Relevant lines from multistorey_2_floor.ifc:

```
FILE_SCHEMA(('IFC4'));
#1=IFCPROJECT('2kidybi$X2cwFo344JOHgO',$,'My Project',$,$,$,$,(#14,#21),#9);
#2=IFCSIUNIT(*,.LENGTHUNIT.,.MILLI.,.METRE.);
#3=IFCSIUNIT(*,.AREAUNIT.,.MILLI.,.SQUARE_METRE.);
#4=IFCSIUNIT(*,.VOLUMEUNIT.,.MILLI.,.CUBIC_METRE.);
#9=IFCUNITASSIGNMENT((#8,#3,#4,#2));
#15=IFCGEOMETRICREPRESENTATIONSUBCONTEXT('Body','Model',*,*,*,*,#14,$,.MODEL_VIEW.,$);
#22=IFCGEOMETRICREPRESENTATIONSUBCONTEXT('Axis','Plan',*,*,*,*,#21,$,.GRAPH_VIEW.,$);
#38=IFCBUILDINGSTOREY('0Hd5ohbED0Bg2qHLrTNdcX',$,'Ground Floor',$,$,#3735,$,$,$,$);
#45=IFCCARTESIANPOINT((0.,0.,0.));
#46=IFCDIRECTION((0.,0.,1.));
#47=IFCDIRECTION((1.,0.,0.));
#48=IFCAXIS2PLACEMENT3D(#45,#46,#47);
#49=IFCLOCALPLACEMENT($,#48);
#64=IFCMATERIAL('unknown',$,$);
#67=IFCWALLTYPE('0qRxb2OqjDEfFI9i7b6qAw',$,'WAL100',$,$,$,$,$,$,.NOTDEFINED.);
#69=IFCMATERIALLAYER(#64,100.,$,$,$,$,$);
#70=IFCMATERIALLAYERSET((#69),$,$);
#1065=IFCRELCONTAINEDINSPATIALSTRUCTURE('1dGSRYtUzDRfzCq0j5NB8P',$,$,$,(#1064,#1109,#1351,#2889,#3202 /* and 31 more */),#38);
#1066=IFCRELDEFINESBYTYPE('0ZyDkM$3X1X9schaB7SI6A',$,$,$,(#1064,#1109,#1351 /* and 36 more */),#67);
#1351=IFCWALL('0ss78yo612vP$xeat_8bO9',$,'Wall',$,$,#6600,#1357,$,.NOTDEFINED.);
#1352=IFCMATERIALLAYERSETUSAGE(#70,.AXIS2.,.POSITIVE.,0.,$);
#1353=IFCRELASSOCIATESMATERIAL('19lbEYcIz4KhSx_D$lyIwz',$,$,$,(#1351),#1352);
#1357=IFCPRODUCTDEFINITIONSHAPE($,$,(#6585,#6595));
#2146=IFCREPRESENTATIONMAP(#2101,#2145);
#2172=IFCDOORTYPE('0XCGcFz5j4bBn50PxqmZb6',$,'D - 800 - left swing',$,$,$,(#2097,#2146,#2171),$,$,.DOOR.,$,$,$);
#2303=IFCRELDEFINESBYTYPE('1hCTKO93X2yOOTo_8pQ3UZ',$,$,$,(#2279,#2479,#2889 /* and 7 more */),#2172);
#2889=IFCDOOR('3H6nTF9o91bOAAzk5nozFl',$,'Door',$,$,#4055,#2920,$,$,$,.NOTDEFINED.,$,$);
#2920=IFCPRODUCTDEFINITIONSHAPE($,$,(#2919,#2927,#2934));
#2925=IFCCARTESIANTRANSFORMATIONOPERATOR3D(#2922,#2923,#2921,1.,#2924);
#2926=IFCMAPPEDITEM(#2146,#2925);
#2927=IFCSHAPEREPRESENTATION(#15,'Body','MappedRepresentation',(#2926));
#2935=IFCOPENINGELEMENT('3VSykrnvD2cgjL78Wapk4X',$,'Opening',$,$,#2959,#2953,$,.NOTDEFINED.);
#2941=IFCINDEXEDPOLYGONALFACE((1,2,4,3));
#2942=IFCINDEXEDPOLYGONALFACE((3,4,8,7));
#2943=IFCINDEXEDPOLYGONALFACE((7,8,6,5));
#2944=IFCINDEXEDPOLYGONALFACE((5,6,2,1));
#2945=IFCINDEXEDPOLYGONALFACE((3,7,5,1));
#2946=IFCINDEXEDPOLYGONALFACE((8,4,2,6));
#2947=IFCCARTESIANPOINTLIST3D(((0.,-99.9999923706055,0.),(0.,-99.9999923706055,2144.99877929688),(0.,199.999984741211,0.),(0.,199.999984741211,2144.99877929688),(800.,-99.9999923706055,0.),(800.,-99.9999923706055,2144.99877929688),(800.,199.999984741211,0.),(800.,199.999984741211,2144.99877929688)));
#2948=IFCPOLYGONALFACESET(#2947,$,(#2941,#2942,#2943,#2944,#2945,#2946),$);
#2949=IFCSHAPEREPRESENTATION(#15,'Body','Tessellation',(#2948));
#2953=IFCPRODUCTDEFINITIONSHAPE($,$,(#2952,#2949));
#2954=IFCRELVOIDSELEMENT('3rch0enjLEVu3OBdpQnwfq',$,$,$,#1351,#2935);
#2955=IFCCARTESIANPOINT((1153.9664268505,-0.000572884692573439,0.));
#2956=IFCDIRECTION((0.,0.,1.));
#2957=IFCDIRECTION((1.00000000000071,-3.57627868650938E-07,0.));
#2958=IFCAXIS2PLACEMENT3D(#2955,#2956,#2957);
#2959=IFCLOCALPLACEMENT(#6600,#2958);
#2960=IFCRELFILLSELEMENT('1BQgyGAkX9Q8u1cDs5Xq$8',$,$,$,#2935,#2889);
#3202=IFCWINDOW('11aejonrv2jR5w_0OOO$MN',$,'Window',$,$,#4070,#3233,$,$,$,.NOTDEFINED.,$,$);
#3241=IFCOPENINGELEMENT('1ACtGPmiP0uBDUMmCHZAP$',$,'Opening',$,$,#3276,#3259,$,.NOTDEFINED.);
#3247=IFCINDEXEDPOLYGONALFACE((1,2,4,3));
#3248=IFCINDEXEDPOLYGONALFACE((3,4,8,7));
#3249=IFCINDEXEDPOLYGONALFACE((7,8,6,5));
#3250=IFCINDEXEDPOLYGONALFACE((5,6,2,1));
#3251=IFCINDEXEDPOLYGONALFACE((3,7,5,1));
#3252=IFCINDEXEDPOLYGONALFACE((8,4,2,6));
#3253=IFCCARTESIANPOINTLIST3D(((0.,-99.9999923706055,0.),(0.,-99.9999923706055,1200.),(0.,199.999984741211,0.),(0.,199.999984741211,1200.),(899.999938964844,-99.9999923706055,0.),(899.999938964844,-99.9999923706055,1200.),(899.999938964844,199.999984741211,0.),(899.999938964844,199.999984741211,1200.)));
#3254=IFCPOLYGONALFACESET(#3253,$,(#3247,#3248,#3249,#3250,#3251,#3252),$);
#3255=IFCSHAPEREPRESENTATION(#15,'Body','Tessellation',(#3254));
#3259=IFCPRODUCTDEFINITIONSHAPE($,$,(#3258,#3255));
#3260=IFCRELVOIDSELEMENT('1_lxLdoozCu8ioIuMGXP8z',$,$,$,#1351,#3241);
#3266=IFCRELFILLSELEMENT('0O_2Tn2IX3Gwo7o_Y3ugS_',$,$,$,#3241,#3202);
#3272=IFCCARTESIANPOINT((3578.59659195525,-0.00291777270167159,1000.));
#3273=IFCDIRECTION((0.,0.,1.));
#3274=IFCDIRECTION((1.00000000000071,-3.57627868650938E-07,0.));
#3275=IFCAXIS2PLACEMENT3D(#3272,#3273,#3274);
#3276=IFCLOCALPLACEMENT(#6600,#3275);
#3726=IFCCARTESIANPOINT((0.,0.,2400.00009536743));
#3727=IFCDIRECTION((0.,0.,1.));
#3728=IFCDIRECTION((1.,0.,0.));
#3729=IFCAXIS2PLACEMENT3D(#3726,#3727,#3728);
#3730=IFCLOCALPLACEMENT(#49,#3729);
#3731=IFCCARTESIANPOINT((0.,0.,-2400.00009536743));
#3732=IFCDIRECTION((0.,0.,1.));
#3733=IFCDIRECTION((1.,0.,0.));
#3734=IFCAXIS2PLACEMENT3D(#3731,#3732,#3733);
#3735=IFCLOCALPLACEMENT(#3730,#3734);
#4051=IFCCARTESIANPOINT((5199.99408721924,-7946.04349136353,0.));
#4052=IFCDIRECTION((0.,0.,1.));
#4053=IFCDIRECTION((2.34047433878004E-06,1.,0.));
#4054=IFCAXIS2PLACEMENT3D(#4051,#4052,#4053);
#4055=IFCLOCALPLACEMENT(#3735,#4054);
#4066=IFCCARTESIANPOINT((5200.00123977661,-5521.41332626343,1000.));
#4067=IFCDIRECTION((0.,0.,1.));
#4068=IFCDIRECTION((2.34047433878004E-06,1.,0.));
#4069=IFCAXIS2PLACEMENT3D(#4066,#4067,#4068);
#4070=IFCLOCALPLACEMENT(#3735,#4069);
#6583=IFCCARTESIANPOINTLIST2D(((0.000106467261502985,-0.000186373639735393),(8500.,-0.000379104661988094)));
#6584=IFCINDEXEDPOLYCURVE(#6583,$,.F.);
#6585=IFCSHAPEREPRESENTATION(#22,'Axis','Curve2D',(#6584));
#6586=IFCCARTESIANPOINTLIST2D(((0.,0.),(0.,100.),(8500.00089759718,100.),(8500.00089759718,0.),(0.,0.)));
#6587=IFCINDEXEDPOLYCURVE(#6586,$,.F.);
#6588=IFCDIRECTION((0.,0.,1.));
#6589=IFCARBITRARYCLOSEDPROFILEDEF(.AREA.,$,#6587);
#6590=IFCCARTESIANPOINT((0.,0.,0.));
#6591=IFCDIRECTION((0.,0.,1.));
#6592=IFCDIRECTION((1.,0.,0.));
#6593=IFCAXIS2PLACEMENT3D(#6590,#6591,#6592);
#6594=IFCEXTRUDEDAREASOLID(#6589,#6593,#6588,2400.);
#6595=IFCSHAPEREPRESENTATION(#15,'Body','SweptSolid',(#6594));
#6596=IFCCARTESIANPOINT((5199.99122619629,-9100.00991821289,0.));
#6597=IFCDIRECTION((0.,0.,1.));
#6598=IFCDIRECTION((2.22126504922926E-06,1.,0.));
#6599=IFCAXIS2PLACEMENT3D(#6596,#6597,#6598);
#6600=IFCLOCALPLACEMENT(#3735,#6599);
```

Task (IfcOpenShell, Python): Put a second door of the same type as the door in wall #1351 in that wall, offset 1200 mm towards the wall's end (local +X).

```python
import ifcopenshell
import ifcopenshell.api.feature
import ifcopenshell.api.geometry
import ifcopenshell.api.root
import ifcopenshell.geom
import ifcopenshell.util.element
import ifcopenshell.util.placement
import ifcopenshell.util.shape
import ifcopenshell.util.unit

model = ifcopenshell.open("multistorey_2_floor.ifc")
unit_scale = ifcopenshell.util.unit.calculate_unit_scale(model)
settings = ifcopenshell.geom.settings()


def volume(element):
    """Net volume in cubic metres, openings subtracted."""
    shape = ifcopenshell.geom.create_shape(settings, element)
    return ifcopenshell.util.shape.get_volume(shape.geometry)


door = model.by_guid("3H6nTF9o91bOAAzk5nozFl")
opening = door.FillsVoids[0].RelatingOpeningElement
wall = opening.VoidsElements[0].RelatingBuildingElement
before = volume(wall)
shift = ifcopenshell.util.placement.get_local_placement(wall.ObjectPlacement)[:3, 0] * 1.2 / unit_scale

# copy_class copies the void relationship, type, container and properties, but no geometry.
new_opening = ifcopenshell.api.root.copy_class(model, product=opening)
new_opening.Representation = ifcopenshell.util.element.copy_deep(
    model, opening.Representation, exclude=["IfcGeometricRepresentationContext", "IfcRepresentationMap"]
)
new_door = ifcopenshell.api.root.copy_class(model, product=door)
new_door.Representation = ifcopenshell.util.element.copy_deep(
    model, door.Representation, exclude=["IfcGeometricRepresentationContext", "IfcRepresentationMap"]
)
ifcopenshell.api.feature.add_filling(model, opening=new_opening, element=new_door)

for old, new in ((opening, new_opening), (door, new_door)):
    matrix = ifcopenshell.util.placement.get_local_placement(old.ObjectPlacement)
    matrix[:3, 3] += shift
    ifcopenshell.api.geometry.edit_object_placement(model, product=new, matrix=matrix, is_si=False)

after = volume(wall)

print(f"wall volume {before:.3f} -> {after:.3f} m3")

model.write("multistorey_2_floor_edited.ifc")
```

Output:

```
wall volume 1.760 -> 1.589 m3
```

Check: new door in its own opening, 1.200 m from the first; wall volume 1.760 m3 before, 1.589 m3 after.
